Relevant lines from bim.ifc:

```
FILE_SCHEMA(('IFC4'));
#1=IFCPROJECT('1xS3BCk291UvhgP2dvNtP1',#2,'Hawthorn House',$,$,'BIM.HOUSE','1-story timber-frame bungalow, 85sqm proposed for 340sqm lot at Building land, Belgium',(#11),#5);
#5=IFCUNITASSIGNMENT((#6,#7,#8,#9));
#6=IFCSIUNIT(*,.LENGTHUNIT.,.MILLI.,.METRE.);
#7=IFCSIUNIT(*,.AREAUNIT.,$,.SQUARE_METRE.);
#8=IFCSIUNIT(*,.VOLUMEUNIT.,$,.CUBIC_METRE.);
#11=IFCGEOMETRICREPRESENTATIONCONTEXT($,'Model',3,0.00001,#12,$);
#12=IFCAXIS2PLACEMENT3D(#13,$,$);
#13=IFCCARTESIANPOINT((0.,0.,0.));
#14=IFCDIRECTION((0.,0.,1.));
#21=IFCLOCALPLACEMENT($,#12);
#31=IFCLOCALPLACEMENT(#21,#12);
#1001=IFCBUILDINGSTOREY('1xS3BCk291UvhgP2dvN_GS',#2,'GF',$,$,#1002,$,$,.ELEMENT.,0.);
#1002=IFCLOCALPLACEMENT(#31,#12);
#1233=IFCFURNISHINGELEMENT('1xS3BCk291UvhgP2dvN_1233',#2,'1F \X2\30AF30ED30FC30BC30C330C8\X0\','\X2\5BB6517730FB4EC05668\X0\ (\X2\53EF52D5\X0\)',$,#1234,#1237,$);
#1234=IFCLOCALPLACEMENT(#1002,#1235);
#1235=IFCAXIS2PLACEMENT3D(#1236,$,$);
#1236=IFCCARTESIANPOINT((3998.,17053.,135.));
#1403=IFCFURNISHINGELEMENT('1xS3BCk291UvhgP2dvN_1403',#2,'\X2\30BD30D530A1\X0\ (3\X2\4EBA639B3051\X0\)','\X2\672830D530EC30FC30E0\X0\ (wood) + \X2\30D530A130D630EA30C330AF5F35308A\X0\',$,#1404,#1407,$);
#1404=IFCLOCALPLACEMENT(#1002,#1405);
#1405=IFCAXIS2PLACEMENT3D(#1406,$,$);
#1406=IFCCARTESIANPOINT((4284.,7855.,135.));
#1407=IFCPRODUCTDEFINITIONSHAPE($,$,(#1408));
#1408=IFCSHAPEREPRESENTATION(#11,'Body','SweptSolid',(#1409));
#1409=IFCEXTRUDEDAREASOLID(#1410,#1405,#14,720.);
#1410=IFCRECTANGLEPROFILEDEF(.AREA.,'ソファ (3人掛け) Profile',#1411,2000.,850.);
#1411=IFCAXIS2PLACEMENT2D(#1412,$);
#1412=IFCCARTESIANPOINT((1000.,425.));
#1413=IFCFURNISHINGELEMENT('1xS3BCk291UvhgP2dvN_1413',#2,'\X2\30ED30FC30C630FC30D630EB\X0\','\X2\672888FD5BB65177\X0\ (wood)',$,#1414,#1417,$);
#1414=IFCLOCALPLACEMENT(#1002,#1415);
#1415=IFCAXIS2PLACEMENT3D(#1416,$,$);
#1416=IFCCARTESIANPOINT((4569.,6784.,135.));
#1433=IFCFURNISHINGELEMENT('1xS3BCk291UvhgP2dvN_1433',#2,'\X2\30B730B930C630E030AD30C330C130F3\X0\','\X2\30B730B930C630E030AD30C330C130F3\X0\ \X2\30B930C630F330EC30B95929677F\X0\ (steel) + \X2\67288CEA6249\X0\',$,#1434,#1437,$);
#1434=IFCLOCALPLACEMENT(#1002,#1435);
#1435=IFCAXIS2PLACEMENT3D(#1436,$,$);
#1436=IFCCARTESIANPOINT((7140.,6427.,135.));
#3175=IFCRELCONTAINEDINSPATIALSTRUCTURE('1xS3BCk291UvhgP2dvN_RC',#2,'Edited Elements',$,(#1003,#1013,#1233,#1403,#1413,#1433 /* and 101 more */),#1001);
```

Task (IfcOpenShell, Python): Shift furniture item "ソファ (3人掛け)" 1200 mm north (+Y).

```python
import ifcopenshell
import ifcopenshell.api.geometry
import ifcopenshell.util.placement
import ifcopenshell.util.unit

model = ifcopenshell.open("bim.ifc")
unit_scale = ifcopenshell.util.unit.calculate_unit_scale(model)

item = model.by_id(1403)
matrix = ifcopenshell.util.placement.get_local_placement(item.ObjectPlacement)
matrix[1, 3] += 1.2 / unit_scale
ifcopenshell.api.geometry.edit_object_placement(model, product=item, matrix=matrix, is_si=False)

print(ifcopenshell.util.placement.get_local_placement(item.ObjectPlacement).round(3) + 0.0)

model.write("bim_updated.ifc")
```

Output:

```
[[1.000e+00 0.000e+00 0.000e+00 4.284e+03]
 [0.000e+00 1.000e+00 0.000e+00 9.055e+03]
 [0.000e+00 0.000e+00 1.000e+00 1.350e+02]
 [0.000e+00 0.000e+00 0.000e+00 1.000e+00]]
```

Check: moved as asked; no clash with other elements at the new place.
